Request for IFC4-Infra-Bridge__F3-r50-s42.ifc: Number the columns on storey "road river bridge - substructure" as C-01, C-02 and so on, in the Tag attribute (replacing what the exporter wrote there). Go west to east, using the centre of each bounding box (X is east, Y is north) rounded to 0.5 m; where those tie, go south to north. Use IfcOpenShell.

First a look at what the model holds.

```python
import ifcopenshell
import ifcopenshell.util.element
import ifcopenshell.util.placement

model = ifcopenshell.open("IFC4-Infra-Bridge__F3-r50-s42.ifc")
print(model.schema)
storey = next(s for s in model.by_type("IfcBuildingStorey") if s.Name == "road river bridge - substructure")
columns = [e for e in ifcopenshell.util.element.get_decomposition(storey) if e.is_a("IfcColumn")]
for e in sorted(columns, key=lambda e: e.id()):
    origin = ifcopenshell.util.placement.get_local_placement(e.ObjectPlacement)[:3, 3]
    print(e.id(), e.Tag, e.Name, origin.round(2) + 0.0, sep=" | ")
```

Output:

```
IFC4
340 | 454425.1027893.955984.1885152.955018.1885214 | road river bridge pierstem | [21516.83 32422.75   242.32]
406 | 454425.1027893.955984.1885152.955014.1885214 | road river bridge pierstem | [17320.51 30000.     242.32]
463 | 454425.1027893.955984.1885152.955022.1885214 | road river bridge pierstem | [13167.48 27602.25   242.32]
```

```python
import ifcopenshell
import ifcopenshell.geom
import ifcopenshell.util.element
import ifcopenshell.util.shape

model = ifcopenshell.open("IFC4-Infra-Bridge__F3-r50-s42.ifc")
settings = ifcopenshell.geom.settings()
settings.set("use-world-coords", True)


def centre(element):
    shape = ifcopenshell.geom.create_shape(settings, element)
    return ifcopenshell.util.shape.get_bbox_centroid(shape.geometry)


storey = next(s for s in model.by_type("IfcBuildingStorey") if s.Name == "road river bridge - substructure")
columns = [e for e in ifcopenshell.util.element.get_decomposition(storey) if e.is_a("IfcColumn")]

# Insertion points can sit at a corner or the storey origin, so sort by the geometry (in metres).
centres = {e: centre(e) for e in columns}
columns.sort(key=lambda e: (round(centres[e][0] / 0.5), centres[e][1]))

for i, e in enumerate(columns, start=1):
    number = f"C-{i:02d}"
    e.Tag = number
    print(e.id(), number)

model.write("IFC4-Infra-Bridge__F3-r50-s42_v2.ifc")
```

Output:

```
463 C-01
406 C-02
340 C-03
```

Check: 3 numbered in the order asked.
